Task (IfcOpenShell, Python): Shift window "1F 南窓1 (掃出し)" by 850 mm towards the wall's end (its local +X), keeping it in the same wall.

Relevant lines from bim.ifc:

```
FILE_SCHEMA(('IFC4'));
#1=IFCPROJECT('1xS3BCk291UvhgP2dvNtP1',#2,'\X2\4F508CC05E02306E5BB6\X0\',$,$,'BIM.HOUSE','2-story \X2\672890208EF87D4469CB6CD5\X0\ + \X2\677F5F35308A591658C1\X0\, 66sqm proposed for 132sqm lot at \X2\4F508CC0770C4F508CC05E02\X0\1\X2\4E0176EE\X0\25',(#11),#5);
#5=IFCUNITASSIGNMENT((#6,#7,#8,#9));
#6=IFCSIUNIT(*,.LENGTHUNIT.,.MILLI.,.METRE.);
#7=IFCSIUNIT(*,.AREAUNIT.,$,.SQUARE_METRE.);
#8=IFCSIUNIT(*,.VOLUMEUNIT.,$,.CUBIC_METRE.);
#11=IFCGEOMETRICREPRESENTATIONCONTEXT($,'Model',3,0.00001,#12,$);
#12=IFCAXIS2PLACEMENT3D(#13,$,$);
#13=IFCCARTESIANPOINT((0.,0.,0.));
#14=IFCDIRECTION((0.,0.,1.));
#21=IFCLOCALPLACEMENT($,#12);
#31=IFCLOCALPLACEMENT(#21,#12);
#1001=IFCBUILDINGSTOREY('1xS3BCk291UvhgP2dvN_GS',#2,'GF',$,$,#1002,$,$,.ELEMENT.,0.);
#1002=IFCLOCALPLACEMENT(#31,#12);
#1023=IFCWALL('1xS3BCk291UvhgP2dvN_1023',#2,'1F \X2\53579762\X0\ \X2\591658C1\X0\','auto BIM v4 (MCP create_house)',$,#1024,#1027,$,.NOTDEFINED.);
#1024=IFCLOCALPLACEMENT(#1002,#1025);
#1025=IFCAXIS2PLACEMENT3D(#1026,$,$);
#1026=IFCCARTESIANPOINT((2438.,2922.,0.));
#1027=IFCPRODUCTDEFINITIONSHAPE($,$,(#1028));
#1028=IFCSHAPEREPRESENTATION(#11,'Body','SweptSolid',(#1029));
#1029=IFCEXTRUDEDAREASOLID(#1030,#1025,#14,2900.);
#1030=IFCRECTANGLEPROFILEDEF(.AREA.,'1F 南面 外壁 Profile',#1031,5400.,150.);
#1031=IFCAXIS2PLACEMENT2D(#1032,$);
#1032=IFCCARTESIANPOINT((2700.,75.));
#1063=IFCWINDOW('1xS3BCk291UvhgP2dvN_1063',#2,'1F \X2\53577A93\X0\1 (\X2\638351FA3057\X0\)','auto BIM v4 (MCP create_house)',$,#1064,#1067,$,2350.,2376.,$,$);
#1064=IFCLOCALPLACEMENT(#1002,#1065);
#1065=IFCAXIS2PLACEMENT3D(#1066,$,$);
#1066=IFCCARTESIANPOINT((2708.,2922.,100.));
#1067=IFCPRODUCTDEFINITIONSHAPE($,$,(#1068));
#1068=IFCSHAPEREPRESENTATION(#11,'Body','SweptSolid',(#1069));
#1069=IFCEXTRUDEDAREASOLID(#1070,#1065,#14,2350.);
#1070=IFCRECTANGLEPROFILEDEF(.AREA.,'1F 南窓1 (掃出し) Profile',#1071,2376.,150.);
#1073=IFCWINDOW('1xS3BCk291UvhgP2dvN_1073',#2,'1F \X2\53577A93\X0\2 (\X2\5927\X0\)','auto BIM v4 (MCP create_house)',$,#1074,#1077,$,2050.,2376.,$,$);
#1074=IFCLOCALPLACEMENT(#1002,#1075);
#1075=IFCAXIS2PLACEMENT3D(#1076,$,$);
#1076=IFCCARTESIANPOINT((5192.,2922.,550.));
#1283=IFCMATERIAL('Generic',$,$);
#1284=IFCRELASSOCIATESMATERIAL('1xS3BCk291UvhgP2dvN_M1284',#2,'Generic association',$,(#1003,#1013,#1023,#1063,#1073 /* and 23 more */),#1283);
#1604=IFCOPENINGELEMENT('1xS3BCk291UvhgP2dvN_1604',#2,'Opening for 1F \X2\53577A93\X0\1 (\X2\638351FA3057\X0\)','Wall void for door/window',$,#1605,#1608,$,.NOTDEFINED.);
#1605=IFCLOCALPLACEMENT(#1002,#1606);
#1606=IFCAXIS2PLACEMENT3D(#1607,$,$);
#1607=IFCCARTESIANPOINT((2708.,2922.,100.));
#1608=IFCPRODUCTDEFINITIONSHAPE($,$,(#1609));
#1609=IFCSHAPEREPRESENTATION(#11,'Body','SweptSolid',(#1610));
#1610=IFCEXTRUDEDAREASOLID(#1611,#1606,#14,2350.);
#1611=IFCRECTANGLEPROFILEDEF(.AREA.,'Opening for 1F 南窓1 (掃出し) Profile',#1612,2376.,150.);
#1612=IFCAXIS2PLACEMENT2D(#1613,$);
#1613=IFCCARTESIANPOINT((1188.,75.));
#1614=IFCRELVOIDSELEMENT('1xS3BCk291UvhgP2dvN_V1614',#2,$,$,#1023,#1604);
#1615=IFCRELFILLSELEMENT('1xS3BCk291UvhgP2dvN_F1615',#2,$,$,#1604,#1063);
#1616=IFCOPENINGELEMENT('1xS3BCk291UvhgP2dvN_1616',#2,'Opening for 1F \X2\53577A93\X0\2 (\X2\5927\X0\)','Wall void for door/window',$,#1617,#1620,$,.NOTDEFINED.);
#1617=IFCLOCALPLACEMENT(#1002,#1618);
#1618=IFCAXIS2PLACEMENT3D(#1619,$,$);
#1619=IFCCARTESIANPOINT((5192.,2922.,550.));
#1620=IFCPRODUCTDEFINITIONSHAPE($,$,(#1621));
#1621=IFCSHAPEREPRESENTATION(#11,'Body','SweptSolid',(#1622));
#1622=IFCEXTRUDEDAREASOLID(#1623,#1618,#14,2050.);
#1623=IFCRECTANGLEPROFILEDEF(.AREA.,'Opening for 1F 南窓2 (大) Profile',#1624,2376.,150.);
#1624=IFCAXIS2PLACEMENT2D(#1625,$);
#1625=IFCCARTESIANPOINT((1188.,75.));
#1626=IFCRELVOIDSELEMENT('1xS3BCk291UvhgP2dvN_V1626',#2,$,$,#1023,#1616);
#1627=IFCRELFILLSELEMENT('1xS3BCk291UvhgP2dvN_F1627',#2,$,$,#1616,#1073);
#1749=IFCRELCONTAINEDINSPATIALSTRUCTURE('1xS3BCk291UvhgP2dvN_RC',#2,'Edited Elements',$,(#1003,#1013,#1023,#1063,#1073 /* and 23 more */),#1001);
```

```python
import ifcopenshell
import ifcopenshell.api.geometry
import ifcopenshell.util.placement
import ifcopenshell.util.unit

model = ifcopenshell.open("bim.ifc")
unit_scale = ifcopenshell.util.unit.calculate_unit_scale(model)

window = model.by_guid("1xS3BCk291UvhgP2dvN_1063")
opening = window.FillsVoids[0].RelatingOpeningElement
wall = opening.VoidsElements[0].RelatingBuildingElement

wall_matrix = ifcopenshell.util.placement.get_local_placement(wall.ObjectPlacement)
shift = wall_matrix[:3, 0] * 0.85 / unit_scale
before = ifcopenshell.util.placement.get_local_placement(window.ObjectPlacement)[:3, 3].copy()

# The window is not placed relative to its opening, so move both.
for product in (opening, window):
    matrix = ifcopenshell.util.placement.get_local_placement(product.ObjectPlacement)
    matrix[:3, 3] += shift
    ifcopenshell.api.geometry.edit_object_placement(model, product=product, matrix=matrix, is_si=False)

after = ifcopenshell.util.placement.get_local_placement(window.ObjectPlacement)[:3, 3]
print("window moved by", (after - before).round(3) + 0.0)

model.write("bim_v2.ifc")
```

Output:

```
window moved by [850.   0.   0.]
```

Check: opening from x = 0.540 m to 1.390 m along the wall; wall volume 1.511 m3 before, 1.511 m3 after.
